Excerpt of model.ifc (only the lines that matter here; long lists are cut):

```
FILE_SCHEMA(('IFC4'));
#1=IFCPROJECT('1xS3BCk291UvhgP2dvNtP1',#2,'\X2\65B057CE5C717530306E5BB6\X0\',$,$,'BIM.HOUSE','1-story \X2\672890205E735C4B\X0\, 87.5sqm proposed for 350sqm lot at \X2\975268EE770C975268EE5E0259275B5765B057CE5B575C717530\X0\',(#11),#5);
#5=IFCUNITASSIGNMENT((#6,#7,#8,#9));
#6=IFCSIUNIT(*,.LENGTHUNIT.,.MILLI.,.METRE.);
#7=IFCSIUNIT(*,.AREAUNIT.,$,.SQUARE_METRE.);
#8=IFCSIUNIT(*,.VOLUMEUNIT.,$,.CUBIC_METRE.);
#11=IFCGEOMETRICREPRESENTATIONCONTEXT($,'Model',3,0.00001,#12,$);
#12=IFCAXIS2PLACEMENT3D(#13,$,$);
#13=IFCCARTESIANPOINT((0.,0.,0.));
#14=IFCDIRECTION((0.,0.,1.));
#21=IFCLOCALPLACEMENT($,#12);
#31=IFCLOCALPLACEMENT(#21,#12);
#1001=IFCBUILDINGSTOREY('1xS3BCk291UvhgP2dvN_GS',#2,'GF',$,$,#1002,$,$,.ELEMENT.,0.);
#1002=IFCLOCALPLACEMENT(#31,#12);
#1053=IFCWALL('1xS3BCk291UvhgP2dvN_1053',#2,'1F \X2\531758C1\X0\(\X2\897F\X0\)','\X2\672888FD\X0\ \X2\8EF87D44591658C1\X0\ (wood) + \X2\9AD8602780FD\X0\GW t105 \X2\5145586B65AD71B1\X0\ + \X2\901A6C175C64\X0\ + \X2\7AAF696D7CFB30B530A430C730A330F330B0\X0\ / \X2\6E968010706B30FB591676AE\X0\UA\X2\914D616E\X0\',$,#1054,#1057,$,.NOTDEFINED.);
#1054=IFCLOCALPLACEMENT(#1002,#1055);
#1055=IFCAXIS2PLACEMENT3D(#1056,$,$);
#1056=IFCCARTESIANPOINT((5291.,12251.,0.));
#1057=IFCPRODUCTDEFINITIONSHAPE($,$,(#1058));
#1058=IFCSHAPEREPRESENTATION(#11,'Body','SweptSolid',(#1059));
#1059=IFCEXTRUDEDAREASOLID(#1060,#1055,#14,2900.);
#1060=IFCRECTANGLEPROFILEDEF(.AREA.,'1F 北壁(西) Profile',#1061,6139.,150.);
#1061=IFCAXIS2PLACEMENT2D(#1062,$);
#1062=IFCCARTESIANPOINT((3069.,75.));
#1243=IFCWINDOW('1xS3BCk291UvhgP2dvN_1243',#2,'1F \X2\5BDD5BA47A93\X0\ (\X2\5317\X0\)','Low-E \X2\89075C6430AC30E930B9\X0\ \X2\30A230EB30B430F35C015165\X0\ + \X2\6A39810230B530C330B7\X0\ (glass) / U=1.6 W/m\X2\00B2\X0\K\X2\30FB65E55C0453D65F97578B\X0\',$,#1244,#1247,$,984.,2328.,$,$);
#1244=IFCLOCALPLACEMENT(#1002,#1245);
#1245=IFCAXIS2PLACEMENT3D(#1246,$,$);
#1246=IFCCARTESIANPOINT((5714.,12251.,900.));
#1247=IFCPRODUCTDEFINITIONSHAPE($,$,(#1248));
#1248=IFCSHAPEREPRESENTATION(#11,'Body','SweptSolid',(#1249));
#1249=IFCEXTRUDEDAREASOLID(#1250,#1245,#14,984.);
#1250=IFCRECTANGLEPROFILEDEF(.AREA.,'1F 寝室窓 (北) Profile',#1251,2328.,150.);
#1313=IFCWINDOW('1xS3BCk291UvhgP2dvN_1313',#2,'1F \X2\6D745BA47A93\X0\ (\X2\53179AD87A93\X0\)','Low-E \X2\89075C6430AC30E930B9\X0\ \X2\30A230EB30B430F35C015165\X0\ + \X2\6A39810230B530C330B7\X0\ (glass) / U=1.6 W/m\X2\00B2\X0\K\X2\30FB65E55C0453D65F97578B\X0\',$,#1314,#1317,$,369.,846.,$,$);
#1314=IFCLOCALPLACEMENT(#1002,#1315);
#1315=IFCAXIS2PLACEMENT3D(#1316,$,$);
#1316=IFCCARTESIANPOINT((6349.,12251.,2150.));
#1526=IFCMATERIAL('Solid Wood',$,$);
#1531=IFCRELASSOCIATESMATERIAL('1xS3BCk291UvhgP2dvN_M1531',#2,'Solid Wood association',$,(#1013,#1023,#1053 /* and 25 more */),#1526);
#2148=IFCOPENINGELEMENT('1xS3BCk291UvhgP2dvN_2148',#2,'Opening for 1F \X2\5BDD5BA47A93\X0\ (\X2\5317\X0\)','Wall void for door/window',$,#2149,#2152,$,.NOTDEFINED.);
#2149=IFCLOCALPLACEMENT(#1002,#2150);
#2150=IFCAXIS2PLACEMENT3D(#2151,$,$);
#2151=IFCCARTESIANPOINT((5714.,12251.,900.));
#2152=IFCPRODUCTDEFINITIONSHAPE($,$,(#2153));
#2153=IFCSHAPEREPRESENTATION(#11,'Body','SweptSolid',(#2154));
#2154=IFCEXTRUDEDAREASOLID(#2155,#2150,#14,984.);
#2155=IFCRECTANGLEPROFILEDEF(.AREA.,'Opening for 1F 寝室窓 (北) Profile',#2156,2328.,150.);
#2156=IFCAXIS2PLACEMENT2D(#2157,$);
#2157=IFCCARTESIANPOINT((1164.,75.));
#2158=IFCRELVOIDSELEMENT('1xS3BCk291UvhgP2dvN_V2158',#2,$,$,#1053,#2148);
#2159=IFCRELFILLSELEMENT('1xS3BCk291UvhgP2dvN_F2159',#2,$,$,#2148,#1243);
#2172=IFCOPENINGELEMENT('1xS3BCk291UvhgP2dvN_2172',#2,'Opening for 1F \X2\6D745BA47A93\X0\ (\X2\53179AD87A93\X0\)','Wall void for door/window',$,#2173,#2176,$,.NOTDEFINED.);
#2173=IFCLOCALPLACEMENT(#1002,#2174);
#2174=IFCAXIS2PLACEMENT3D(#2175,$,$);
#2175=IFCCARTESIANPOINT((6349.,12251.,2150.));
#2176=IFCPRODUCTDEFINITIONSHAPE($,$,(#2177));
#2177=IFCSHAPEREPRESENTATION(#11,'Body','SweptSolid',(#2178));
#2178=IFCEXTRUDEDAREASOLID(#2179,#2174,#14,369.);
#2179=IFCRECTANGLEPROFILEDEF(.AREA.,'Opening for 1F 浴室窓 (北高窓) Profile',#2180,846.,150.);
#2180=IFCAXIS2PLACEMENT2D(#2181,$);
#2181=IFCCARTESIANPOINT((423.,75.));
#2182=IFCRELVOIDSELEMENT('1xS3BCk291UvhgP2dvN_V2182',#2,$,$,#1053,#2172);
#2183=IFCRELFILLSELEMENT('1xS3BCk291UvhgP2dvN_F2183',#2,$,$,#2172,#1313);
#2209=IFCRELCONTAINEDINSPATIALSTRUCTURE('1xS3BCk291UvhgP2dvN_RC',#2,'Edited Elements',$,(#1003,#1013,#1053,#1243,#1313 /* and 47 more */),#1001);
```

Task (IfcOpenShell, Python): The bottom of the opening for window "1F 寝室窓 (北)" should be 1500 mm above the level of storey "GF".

```python
import numpy as np
import ifcopenshell
import ifcopenshell.api.geometry
import ifcopenshell.geom
import ifcopenshell.util.element
import ifcopenshell.util.placement
import ifcopenshell.util.shape
import ifcopenshell.util.unit

model = ifcopenshell.open("model.ifc")
unit_scale = ifcopenshell.util.unit.calculate_unit_scale(model)

window = model.by_guid("1xS3BCk291UvhgP2dvN_1243")
opening = window.FillsVoids[0].RelatingOpeningElement
storey = ifcopenshell.util.element.get_container(window, ifc_class="IfcBuildingStorey")
level = ifcopenshell.util.placement.get_local_placement(storey.ObjectPlacement)[2, 3]

# The opening's origin need not be at the sill, so measure its lowest point.
shape = ifcopenshell.geom.create_shape(ifcopenshell.geom.settings(), opening)
bottom = ifcopenshell.util.shape.get_shape_bottom_elevation(shape, shape.geometry) / unit_scale
dz = level + 1.5 / unit_scale - bottom

shift = np.array([0.0, 0.0, dz])
# The window is not placed relative to its opening, so move both.
for product in (opening, window):
    matrix = ifcopenshell.util.placement.get_local_placement(product.ObjectPlacement)
    matrix[:3, 3] += shift
    ifcopenshell.api.geometry.edit_object_placement(model, product=product, matrix=matrix, is_si=False)

print(f"moved by {dz * unit_scale:+.3f} m")

model.write("model_updated.ifc")
```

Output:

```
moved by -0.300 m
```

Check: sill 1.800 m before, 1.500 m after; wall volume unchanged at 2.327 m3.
